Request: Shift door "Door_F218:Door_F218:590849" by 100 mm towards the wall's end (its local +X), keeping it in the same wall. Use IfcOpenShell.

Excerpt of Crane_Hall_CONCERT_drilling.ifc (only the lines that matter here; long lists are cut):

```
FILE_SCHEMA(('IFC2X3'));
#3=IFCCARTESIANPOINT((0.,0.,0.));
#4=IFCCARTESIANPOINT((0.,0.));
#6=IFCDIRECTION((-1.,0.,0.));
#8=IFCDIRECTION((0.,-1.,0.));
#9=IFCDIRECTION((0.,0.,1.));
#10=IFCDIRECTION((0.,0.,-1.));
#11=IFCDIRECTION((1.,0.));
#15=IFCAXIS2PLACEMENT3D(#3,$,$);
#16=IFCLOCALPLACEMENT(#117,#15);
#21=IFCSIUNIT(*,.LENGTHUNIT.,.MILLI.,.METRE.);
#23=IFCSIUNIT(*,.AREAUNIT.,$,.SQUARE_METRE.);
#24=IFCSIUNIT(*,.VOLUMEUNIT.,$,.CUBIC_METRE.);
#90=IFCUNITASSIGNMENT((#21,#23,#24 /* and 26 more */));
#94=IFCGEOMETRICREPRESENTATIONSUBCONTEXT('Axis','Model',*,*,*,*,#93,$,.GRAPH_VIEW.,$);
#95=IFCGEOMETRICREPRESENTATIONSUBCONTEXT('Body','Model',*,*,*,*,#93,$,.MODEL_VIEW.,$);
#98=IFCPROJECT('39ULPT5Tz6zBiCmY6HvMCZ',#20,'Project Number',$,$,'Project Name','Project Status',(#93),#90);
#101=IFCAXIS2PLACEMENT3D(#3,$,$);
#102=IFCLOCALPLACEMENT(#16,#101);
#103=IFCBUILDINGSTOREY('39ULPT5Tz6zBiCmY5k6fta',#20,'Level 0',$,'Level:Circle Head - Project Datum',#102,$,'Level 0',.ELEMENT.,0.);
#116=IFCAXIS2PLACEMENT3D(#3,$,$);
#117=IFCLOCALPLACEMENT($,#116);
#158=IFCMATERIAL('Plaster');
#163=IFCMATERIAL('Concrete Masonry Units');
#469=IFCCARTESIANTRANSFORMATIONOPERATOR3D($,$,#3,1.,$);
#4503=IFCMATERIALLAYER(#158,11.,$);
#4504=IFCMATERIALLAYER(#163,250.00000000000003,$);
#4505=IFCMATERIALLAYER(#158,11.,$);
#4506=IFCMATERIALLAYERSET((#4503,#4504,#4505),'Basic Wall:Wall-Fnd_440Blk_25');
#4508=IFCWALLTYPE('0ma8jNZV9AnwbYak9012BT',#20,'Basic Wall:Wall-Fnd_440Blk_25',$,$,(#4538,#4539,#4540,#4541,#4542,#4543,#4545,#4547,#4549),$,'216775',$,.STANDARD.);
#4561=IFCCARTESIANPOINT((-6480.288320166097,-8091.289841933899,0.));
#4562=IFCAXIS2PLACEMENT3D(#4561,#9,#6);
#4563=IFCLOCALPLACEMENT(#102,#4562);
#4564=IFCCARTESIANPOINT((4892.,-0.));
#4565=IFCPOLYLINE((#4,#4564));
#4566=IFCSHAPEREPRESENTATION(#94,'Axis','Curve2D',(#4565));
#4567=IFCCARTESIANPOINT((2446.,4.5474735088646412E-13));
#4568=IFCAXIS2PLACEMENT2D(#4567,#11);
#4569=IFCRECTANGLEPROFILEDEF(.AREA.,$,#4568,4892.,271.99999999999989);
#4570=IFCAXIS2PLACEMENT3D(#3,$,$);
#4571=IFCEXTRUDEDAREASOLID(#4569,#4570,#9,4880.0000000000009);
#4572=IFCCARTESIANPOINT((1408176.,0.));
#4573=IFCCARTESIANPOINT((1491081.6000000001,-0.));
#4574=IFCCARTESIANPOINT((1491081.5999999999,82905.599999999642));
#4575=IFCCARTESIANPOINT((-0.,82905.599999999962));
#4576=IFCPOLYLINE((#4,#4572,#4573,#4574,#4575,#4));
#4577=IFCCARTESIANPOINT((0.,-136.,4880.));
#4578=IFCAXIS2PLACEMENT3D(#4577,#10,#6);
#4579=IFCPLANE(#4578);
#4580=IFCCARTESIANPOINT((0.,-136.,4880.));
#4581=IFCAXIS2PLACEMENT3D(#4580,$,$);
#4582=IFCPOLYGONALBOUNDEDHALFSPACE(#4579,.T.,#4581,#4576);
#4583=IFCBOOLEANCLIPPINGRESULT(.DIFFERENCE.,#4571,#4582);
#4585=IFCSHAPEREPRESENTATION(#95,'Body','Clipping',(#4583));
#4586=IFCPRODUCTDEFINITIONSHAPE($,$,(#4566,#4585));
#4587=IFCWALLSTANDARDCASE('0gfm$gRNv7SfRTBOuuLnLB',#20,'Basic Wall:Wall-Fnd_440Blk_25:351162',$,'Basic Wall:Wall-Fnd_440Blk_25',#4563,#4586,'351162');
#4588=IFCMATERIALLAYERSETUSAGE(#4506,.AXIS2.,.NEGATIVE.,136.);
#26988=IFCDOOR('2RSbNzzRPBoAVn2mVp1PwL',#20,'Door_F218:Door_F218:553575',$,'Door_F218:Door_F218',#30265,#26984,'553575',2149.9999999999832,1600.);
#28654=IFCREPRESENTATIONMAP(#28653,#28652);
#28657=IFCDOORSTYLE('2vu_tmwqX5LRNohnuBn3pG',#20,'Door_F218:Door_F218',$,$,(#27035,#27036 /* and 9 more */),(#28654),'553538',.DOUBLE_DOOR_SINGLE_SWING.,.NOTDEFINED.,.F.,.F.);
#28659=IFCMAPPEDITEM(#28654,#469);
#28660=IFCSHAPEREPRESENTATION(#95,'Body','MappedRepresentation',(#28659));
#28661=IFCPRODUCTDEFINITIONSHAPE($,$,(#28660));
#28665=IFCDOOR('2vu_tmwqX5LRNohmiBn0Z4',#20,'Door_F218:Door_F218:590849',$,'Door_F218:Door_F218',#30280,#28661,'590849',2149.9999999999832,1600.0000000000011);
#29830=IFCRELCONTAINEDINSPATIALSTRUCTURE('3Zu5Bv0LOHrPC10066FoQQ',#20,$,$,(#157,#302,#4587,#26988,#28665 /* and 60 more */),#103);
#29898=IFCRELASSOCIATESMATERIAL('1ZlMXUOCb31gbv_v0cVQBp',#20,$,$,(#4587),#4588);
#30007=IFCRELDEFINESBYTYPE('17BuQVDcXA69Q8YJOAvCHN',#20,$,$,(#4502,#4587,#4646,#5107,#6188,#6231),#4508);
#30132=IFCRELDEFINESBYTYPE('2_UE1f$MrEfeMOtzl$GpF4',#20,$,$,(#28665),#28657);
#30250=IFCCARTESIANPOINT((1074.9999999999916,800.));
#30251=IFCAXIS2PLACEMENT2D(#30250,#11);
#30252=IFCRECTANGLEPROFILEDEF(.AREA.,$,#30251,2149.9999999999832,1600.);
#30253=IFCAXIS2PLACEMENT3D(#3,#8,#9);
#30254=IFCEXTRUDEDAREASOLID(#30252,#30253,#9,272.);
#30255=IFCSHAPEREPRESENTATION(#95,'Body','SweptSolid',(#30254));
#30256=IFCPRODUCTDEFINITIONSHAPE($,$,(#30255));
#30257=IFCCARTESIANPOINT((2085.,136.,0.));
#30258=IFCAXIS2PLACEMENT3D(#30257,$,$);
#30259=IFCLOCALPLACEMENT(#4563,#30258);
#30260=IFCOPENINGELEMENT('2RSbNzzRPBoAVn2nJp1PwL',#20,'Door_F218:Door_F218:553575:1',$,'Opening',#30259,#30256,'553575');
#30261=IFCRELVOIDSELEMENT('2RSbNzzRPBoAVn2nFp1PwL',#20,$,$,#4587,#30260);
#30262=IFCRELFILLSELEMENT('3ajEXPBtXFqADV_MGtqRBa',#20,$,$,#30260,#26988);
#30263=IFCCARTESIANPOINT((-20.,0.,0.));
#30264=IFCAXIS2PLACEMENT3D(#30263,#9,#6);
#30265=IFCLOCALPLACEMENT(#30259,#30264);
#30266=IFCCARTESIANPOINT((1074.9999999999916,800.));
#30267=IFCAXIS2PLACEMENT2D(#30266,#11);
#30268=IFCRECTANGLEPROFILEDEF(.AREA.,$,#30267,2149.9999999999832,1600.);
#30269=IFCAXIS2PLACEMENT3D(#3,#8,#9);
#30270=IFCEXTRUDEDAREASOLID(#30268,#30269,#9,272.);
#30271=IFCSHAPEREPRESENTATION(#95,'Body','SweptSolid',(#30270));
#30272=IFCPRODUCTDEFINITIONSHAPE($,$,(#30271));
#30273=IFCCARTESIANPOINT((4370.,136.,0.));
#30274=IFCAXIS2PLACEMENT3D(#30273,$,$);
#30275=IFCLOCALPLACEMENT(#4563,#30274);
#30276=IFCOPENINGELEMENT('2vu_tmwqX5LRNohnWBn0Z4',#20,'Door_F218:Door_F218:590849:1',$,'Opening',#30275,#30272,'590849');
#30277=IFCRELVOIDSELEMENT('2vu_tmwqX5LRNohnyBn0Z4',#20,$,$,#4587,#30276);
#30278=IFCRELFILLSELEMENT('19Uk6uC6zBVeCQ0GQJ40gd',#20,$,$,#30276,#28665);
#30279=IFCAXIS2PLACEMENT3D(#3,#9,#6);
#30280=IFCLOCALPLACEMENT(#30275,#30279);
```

```python
import ifcopenshell
import ifcopenshell.api.geometry
import ifcopenshell.util.placement

model = ifcopenshell.open("Crane_Hall_CONCERT_drilling.ifc")

door = model.by_guid("2vu_tmwqX5LRNohmiBn0Z4")
opening = door.FillsVoids[0].RelatingOpeningElement
wall = opening.VoidsElements[0].RelatingBuildingElement

wall_matrix = ifcopenshell.util.placement.get_local_placement(wall.ObjectPlacement)
shift = wall_matrix[:3, 0] * 100.0
before = ifcopenshell.util.placement.get_local_placement(door.ObjectPlacement)[:3, 3].copy()

# The door is placed relative to its opening, so it follows when the opening moves.
matrix = ifcopenshell.util.placement.get_local_placement(opening.ObjectPlacement)
matrix[:3, 3] += shift
ifcopenshell.api.geometry.edit_object_placement(
    model, product=opening, matrix=matrix, is_si=False, should_transform_children=True
)

after = ifcopenshell.util.placement.get_local_placement(door.ObjectPlacement)[:3, 3]
print("door moved by", (after - before).round(3) + 0.0)

model.write("Crane_Hall_CONCERT_drilling_v2.ifc")
```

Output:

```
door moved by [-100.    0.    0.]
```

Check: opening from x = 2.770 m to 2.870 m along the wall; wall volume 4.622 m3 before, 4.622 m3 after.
